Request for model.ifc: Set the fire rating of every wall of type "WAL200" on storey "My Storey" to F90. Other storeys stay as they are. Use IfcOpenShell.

First a look at what the model holds.

```python
import ifcopenshell
import ifcopenshell.util.element

model = ifcopenshell.open("model.ifc")
print(model.schema)
storey = next(s for s in model.by_type("IfcBuildingStorey") if s.Name == "My Storey")
walls = [e for e in ifcopenshell.util.element.get_decomposition(storey) if e.is_a("IfcWall")]
seen = {}
for e in walls:
    element_type = ifcopenshell.util.element.get_type(e)
    key = (element_type.Name if element_type != e and element_type else None, ifcopenshell.util.element.get_pset(e, "Pset_WallCommon", "FireRating"))
    seen[key] = seen.get(key, 0) + 1
for (name, value), count in sorted(seen.items(), key=str):
    print(count, "x", name, "|", value)
```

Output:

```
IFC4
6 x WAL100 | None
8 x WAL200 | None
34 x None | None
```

```python
import ifcopenshell
import ifcopenshell.api.pset
import ifcopenshell.util.element

model = ifcopenshell.open("model.ifc")

storey = next(s for s in model.by_type("IfcBuildingStorey") if s.Name == "My Storey")
walls = [e for e in ifcopenshell.util.element.get_decomposition(storey) if e.is_a("IfcWall")]

count = 0
for e in walls:
    element_type = ifcopenshell.util.element.get_type(e)
    if element_type in (None, e) or element_type.Name != "WAL200":
        continue
    # add_pset returns the element's existing set when there is one.
    pset = ifcopenshell.api.pset.add_pset(model, product=e, name="Pset_WallCommon")
    ifcopenshell.api.pset.edit_pset(model, pset=pset, properties={"FireRating": "F90"})
    count += 1

print(count, "walls updated")

model.write("model_rev.ifc")
```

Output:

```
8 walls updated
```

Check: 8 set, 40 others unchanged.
